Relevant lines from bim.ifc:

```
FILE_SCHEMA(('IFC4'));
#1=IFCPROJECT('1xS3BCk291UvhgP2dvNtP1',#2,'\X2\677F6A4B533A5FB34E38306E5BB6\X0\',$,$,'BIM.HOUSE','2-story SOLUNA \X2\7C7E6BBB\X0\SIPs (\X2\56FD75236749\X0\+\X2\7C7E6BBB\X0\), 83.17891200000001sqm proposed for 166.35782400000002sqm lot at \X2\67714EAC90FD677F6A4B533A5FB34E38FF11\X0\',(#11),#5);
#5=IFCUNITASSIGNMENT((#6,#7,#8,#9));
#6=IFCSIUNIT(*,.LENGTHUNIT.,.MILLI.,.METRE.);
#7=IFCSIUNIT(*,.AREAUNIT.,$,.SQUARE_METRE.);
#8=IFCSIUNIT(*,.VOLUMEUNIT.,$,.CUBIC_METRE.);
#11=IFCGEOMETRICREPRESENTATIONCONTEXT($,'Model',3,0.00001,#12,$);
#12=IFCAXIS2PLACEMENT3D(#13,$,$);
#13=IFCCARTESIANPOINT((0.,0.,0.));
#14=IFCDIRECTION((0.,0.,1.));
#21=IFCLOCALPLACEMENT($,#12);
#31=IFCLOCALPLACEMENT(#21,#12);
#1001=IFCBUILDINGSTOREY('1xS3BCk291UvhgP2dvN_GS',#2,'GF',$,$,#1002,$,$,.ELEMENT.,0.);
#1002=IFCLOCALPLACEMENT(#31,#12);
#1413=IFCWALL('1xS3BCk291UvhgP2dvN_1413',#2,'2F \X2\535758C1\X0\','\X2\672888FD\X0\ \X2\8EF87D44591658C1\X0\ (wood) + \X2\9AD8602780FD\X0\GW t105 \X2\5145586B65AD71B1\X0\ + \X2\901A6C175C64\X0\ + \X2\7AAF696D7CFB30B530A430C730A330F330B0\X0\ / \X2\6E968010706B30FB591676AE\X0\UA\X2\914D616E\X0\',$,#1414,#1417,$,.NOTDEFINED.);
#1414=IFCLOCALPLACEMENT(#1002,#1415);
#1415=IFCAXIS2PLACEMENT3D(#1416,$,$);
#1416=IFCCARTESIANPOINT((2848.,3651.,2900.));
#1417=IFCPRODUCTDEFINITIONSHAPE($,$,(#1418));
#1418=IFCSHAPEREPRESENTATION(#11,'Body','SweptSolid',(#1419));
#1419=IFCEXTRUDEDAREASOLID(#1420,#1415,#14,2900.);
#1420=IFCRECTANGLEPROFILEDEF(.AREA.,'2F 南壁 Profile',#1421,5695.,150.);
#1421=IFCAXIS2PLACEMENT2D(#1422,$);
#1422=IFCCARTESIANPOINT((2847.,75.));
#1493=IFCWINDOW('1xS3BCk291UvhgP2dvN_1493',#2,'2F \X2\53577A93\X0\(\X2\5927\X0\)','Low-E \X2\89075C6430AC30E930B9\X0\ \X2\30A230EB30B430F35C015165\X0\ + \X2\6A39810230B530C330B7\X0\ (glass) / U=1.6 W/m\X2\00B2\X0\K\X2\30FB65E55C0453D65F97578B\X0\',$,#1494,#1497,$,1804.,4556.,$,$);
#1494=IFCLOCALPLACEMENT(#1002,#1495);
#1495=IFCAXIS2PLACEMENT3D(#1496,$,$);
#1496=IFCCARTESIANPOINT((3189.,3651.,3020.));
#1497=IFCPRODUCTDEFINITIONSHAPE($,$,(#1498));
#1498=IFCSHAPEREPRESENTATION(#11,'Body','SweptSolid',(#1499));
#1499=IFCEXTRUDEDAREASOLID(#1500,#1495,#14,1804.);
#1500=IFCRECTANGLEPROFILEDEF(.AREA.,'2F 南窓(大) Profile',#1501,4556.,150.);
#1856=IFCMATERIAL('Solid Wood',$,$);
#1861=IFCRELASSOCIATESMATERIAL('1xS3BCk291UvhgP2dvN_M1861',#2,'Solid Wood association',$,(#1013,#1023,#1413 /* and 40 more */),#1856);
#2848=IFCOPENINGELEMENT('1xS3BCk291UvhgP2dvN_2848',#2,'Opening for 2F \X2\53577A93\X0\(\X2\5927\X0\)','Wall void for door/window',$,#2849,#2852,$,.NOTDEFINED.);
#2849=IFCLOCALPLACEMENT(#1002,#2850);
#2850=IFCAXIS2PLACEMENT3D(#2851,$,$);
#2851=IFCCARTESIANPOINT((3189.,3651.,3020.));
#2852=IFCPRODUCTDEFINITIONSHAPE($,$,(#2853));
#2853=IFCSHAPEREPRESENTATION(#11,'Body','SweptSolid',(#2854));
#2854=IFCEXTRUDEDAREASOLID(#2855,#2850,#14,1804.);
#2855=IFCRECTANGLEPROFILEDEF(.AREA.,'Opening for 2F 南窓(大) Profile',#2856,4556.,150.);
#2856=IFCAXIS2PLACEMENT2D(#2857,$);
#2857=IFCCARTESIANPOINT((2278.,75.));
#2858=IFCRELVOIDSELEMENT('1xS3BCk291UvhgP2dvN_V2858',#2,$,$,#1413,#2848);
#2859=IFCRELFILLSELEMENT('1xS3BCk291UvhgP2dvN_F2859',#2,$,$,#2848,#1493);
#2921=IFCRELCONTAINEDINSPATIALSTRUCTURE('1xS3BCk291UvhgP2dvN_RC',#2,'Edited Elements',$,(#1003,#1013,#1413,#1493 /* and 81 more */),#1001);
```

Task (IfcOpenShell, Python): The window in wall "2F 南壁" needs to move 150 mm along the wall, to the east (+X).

```python
import ifcopenshell
import ifcopenshell.api.geometry
import ifcopenshell.util.placement
import ifcopenshell.util.unit

model = ifcopenshell.open("bim.ifc")
unit_scale = ifcopenshell.util.unit.calculate_unit_scale(model)

window = model.by_guid("1xS3BCk291UvhgP2dvN_1493")
opening = window.FillsVoids[0].RelatingOpeningElement
wall = opening.VoidsElements[0].RelatingBuildingElement

wall_matrix = ifcopenshell.util.placement.get_local_placement(wall.ObjectPlacement)
shift = wall_matrix[:3, 0] * 0.15 / unit_scale
before = ifcopenshell.util.placement.get_local_placement(window.ObjectPlacement)[:3, 3].copy()

# The window is not placed relative to its opening, so move both.
for product in (opening, window):
    matrix = ifcopenshell.util.placement.get_local_placement(product.ObjectPlacement)
    matrix[:3, 3] += shift
    ifcopenshell.api.geometry.edit_object_placement(model, product=product, matrix=matrix, is_si=False)

after = ifcopenshell.util.placement.get_local_placement(window.ObjectPlacement)[:3, 3]
print("window moved by", (after - before).round(3) + 0.0)

model.write("bim_updated.ifc")
```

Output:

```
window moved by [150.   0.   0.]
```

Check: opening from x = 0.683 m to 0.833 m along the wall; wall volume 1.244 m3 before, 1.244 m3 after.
